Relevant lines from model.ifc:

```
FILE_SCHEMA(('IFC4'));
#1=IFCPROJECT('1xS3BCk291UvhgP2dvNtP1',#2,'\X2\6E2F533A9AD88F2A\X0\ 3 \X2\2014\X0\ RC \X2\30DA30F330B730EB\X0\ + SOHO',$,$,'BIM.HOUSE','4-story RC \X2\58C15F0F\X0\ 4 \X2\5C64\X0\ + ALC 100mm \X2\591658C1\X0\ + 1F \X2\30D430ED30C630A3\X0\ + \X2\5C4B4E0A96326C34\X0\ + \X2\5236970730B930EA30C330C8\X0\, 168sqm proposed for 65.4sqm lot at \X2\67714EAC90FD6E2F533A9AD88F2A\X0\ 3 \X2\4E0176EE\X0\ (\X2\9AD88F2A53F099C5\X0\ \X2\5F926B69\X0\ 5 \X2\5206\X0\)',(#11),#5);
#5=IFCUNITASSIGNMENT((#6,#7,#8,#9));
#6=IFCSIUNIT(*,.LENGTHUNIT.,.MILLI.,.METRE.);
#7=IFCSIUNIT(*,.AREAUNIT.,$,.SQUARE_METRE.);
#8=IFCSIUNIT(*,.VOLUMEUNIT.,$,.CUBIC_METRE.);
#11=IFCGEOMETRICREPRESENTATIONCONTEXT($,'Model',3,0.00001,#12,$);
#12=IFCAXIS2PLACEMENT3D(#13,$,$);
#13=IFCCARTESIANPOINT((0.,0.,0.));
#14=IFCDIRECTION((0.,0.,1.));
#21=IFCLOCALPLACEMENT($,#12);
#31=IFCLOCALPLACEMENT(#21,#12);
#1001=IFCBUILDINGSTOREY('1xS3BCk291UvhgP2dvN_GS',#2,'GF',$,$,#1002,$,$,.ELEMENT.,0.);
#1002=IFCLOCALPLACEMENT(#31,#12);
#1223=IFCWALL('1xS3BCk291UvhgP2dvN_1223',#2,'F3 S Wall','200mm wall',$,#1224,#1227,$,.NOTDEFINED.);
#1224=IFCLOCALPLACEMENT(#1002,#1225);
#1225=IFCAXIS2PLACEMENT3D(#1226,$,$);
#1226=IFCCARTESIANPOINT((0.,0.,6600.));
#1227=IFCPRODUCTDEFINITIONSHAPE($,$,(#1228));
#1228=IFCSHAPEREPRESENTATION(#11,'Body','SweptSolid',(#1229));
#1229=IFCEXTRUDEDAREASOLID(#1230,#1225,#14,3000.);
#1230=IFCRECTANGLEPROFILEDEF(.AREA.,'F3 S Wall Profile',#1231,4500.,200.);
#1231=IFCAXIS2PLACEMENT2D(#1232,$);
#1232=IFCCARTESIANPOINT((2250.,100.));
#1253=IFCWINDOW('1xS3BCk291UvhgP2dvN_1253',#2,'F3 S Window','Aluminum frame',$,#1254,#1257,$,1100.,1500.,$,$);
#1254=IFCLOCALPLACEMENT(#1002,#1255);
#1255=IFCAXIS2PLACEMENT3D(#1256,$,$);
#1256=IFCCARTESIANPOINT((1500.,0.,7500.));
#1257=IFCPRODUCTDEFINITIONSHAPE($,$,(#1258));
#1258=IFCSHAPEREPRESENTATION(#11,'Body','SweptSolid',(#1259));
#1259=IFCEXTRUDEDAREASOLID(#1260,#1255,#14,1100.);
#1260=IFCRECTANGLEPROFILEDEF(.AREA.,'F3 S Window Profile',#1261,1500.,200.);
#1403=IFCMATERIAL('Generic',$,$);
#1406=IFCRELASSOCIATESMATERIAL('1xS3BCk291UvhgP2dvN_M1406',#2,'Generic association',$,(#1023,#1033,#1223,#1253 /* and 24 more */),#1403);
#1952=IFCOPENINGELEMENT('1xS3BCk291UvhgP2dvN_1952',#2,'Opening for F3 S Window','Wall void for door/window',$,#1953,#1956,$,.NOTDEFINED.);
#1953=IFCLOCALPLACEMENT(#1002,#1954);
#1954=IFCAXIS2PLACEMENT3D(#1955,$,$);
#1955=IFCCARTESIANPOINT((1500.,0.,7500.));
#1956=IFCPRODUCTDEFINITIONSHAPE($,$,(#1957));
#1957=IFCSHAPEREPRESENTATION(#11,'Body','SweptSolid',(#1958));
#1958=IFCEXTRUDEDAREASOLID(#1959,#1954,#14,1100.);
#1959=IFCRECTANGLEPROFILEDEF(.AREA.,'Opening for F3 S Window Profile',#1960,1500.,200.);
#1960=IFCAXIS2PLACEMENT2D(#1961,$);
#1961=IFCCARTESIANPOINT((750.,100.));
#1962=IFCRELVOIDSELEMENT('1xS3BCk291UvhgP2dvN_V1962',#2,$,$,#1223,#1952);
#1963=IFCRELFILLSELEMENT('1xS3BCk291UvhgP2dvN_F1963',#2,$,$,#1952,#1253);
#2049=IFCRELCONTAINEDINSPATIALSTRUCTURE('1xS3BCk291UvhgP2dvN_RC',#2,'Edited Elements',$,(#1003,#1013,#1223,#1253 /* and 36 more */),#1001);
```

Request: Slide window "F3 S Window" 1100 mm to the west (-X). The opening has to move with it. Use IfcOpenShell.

```python
import ifcopenshell
import ifcopenshell.api.geometry
import ifcopenshell.util.placement

model = ifcopenshell.open("model.ifc")

window = model.by_guid("1xS3BCk291UvhgP2dvN_1253")
opening = window.FillsVoids[0].RelatingOpeningElement
wall = opening.VoidsElements[0].RelatingBuildingElement

wall_matrix = ifcopenshell.util.placement.get_local_placement(wall.ObjectPlacement)
shift = wall_matrix[:3, 0] * -1100.0
before = ifcopenshell.util.placement.get_local_placement(window.ObjectPlacement)[:3, 3].copy()

# The window is not placed relative to its opening, so move both.
for product in (opening, window):
    matrix = ifcopenshell.util.placement.get_local_placement(product.ObjectPlacement)
    matrix[:3, 3] += shift
    ifcopenshell.api.geometry.edit_object_placement(model, product=product, matrix=matrix, is_si=False)

after = ifcopenshell.util.placement.get_local_placement(window.ObjectPlacement)[:3, 3]
print("window moved by", (after - before).round(3) + 0.0)

model.write("model_v2.ifc")
```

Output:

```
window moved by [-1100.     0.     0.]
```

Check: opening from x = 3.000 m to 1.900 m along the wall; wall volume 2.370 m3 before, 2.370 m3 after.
